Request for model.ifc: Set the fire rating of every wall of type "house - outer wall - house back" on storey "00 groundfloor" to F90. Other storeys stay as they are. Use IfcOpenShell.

First a look at what the model holds.

```python
import ifcopenshell
import ifcopenshell.util.element

model = ifcopenshell.open("model.ifc")
print(model.schema)
storey = next(s for s in model.by_type("IfcBuildingStorey") if s.Name == "00 groundfloor")
walls = [e for e in ifcopenshell.util.element.get_decomposition(storey) if e.is_a("IfcWall")]
seen = {}
for e in walls:
    element_type = ifcopenshell.util.element.get_type(e)
    key = (element_type.Name if element_type != e and element_type else None, ifcopenshell.util.element.get_pset(e, "Pset_WallCommon", "FireRating"))
    seen[key] = seen.get(key, 0) + 1
for (name, value), count in sorted(seen.items(), key=str):
    print(count, "x", name, "|", value)
```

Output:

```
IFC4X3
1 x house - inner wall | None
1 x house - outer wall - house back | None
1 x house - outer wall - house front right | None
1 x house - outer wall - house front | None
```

```python
import ifcopenshell
import ifcopenshell.api.pset
import ifcopenshell.util.element

model = ifcopenshell.open("model.ifc")

storey = next(s for s in model.by_type("IfcBuildingStorey") if s.Name == "00 groundfloor")
walls = [e for e in ifcopenshell.util.element.get_decomposition(storey) if e.is_a("IfcWall")]

count = 0
for e in walls:
    element_type = ifcopenshell.util.element.get_type(e)
    if element_type in (None, e) or element_type.Name != "house - outer wall - house back":
        continue
    # add_pset returns the element's existing set when there is one.
    pset = ifcopenshell.api.pset.add_pset(model, product=e, name="Pset_WallCommon")
    ifcopenshell.api.pset.edit_pset(model, pset=pset, properties={"FireRating": "F90"})
    count += 1

print(count, "walls updated")

model.write("model_edited.ifc")
```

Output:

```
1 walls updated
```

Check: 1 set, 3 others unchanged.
